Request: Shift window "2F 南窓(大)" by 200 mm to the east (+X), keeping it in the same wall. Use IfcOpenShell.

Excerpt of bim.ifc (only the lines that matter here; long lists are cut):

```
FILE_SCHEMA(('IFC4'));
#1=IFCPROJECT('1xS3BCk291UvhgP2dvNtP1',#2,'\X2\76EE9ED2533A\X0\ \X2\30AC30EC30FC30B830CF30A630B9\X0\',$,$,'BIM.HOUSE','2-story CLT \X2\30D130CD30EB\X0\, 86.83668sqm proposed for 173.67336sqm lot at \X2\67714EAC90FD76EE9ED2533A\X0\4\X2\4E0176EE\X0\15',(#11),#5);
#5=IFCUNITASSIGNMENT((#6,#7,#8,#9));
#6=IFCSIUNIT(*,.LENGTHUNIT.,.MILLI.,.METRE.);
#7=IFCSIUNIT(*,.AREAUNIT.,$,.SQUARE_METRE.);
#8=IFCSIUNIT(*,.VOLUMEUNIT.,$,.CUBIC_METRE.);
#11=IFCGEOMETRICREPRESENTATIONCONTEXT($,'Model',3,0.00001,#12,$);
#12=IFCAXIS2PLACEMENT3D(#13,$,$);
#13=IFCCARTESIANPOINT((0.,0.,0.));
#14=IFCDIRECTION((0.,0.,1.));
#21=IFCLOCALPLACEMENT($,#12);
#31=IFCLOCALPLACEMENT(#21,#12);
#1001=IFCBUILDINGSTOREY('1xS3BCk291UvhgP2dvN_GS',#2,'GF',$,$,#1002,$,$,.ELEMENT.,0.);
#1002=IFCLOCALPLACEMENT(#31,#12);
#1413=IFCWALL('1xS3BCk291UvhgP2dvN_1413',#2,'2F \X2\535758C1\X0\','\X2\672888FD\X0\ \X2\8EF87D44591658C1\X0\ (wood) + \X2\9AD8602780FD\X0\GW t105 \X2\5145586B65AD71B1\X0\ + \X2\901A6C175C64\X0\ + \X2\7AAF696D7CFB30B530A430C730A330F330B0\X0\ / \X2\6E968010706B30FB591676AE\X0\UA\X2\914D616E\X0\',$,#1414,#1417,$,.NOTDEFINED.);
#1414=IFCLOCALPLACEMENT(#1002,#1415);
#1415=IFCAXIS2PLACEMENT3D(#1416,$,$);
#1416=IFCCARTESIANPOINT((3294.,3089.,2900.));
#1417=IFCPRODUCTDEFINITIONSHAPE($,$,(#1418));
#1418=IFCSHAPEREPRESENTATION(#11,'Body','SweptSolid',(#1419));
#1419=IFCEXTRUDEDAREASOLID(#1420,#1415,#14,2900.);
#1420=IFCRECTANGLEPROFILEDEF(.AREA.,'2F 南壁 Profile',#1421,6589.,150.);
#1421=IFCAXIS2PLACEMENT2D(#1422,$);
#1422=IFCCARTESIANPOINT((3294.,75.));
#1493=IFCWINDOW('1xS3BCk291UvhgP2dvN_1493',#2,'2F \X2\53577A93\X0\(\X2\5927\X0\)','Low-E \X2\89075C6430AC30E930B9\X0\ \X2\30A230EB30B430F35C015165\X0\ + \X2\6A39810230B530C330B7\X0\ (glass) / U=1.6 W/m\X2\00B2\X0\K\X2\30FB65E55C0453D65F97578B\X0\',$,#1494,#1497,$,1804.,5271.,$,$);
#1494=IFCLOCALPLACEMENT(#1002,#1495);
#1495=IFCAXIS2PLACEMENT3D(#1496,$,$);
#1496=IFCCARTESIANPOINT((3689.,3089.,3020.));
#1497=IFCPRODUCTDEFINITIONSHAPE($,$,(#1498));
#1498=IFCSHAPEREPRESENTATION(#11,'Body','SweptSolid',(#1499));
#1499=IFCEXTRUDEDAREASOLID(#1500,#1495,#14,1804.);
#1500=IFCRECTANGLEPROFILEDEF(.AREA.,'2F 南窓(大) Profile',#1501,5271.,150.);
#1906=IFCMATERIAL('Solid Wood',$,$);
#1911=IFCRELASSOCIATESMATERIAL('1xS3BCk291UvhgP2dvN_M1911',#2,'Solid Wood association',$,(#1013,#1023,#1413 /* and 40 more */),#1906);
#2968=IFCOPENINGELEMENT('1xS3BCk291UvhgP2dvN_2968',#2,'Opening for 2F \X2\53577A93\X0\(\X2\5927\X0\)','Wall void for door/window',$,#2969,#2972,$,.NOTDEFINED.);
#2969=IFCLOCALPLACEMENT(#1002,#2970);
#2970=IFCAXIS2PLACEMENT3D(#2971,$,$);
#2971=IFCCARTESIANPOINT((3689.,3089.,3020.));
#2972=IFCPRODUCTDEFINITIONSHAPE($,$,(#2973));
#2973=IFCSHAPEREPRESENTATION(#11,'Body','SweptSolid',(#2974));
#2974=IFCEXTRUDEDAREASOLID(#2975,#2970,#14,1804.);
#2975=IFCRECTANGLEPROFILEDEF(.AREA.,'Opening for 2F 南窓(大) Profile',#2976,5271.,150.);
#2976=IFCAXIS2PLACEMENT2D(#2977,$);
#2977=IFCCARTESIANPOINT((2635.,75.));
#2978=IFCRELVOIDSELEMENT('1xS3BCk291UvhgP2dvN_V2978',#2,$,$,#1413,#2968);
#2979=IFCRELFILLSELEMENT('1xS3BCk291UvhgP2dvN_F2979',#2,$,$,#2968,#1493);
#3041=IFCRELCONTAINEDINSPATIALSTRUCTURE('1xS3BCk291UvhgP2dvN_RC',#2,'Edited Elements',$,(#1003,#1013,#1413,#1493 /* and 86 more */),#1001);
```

```python
import ifcopenshell
import ifcopenshell.api.geometry
import ifcopenshell.util.placement
import ifcopenshell.util.unit

model = ifcopenshell.open("bim.ifc")
unit_scale = ifcopenshell.util.unit.calculate_unit_scale(model)

window = model.by_guid("1xS3BCk291UvhgP2dvN_1493")
opening = window.FillsVoids[0].RelatingOpeningElement
wall = opening.VoidsElements[0].RelatingBuildingElement

wall_matrix = ifcopenshell.util.placement.get_local_placement(wall.ObjectPlacement)
shift = wall_matrix[:3, 0] * 0.2 / unit_scale
before = ifcopenshell.util.placement.get_local_placement(window.ObjectPlacement)[:3, 3].copy()

# The window is not placed relative to its opening, so move both.
for product in (opening, window):
    matrix = ifcopenshell.util.placement.get_local_placement(product.ObjectPlacement)
    matrix[:3, 3] += shift
    ifcopenshell.api.geometry.edit_object_placement(model, product=product, matrix=matrix, is_si=False)

after = ifcopenshell.util.placement.get_local_placement(window.ObjectPlacement)[:3, 3]
print("window moved by", (after - before).round(3) + 0.0)

model.write("bim_updated.ifc")
```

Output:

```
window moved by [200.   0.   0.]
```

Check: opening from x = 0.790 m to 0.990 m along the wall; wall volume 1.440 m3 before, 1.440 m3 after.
